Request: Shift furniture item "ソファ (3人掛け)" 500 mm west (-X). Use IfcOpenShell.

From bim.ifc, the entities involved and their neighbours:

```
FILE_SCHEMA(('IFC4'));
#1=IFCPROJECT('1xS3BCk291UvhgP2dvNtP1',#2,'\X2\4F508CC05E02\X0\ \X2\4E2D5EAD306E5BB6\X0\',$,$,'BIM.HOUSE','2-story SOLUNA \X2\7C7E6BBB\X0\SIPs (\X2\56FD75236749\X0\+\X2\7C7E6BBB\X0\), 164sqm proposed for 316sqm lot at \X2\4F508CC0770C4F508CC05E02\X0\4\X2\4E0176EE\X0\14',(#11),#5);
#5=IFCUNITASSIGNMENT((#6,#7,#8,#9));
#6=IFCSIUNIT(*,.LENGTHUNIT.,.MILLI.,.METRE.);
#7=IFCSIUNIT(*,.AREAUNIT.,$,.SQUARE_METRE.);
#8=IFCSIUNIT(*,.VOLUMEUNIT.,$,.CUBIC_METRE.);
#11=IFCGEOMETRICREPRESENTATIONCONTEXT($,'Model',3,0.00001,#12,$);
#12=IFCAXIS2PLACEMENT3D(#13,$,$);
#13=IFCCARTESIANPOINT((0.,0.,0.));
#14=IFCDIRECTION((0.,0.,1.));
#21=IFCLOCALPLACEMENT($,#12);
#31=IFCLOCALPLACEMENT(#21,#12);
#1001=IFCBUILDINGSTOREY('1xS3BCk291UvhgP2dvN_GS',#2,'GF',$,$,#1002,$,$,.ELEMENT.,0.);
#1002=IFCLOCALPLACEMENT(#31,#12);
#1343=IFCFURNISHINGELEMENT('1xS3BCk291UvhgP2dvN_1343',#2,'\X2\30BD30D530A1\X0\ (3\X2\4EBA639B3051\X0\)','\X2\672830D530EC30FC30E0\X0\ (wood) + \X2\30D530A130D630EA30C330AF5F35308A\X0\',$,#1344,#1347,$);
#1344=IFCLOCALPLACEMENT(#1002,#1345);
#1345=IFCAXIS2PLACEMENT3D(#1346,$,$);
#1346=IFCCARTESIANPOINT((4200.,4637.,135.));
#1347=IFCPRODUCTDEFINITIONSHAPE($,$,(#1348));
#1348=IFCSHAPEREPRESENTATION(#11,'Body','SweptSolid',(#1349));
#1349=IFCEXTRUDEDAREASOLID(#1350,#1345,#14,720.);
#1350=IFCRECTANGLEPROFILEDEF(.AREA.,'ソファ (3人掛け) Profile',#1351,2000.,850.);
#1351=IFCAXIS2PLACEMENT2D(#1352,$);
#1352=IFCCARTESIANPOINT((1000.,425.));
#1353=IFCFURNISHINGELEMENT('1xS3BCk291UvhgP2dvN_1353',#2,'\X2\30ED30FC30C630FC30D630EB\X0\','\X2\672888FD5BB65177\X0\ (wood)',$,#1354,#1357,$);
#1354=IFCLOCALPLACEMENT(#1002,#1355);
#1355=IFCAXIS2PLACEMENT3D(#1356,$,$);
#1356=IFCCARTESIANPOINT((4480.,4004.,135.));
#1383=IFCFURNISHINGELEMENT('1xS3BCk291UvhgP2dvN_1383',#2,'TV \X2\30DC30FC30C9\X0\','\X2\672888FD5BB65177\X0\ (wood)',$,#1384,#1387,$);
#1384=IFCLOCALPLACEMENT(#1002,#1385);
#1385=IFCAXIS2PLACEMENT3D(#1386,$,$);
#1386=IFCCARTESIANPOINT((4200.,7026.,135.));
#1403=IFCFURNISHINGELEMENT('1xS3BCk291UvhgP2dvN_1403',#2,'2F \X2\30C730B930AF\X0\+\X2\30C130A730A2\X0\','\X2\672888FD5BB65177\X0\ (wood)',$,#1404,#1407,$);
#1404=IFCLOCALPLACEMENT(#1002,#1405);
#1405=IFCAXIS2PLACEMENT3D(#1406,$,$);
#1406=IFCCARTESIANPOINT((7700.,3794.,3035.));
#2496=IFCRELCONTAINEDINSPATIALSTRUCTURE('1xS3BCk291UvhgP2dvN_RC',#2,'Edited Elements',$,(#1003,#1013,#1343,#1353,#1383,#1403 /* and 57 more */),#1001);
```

```python
import ifcopenshell
import ifcopenshell.api.geometry
import ifcopenshell.util.placement
import ifcopenshell.util.unit

model = ifcopenshell.open("bim.ifc")
unit_scale = ifcopenshell.util.unit.calculate_unit_scale(model)

item = model.by_guid("1xS3BCk291UvhgP2dvN_1343")
matrix = ifcopenshell.util.placement.get_local_placement(item.ObjectPlacement)
matrix[0, 3] -= 0.5 / unit_scale
ifcopenshell.api.geometry.edit_object_placement(model, product=item, matrix=matrix, is_si=False)

print(ifcopenshell.util.placement.get_local_placement(item.ObjectPlacement).round(3) + 0.0)

model.write("bim-out.ifc")
```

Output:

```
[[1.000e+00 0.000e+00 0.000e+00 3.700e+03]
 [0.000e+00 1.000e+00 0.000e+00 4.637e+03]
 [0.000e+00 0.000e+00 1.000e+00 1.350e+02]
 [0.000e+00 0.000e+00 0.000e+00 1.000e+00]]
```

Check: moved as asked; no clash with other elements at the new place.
